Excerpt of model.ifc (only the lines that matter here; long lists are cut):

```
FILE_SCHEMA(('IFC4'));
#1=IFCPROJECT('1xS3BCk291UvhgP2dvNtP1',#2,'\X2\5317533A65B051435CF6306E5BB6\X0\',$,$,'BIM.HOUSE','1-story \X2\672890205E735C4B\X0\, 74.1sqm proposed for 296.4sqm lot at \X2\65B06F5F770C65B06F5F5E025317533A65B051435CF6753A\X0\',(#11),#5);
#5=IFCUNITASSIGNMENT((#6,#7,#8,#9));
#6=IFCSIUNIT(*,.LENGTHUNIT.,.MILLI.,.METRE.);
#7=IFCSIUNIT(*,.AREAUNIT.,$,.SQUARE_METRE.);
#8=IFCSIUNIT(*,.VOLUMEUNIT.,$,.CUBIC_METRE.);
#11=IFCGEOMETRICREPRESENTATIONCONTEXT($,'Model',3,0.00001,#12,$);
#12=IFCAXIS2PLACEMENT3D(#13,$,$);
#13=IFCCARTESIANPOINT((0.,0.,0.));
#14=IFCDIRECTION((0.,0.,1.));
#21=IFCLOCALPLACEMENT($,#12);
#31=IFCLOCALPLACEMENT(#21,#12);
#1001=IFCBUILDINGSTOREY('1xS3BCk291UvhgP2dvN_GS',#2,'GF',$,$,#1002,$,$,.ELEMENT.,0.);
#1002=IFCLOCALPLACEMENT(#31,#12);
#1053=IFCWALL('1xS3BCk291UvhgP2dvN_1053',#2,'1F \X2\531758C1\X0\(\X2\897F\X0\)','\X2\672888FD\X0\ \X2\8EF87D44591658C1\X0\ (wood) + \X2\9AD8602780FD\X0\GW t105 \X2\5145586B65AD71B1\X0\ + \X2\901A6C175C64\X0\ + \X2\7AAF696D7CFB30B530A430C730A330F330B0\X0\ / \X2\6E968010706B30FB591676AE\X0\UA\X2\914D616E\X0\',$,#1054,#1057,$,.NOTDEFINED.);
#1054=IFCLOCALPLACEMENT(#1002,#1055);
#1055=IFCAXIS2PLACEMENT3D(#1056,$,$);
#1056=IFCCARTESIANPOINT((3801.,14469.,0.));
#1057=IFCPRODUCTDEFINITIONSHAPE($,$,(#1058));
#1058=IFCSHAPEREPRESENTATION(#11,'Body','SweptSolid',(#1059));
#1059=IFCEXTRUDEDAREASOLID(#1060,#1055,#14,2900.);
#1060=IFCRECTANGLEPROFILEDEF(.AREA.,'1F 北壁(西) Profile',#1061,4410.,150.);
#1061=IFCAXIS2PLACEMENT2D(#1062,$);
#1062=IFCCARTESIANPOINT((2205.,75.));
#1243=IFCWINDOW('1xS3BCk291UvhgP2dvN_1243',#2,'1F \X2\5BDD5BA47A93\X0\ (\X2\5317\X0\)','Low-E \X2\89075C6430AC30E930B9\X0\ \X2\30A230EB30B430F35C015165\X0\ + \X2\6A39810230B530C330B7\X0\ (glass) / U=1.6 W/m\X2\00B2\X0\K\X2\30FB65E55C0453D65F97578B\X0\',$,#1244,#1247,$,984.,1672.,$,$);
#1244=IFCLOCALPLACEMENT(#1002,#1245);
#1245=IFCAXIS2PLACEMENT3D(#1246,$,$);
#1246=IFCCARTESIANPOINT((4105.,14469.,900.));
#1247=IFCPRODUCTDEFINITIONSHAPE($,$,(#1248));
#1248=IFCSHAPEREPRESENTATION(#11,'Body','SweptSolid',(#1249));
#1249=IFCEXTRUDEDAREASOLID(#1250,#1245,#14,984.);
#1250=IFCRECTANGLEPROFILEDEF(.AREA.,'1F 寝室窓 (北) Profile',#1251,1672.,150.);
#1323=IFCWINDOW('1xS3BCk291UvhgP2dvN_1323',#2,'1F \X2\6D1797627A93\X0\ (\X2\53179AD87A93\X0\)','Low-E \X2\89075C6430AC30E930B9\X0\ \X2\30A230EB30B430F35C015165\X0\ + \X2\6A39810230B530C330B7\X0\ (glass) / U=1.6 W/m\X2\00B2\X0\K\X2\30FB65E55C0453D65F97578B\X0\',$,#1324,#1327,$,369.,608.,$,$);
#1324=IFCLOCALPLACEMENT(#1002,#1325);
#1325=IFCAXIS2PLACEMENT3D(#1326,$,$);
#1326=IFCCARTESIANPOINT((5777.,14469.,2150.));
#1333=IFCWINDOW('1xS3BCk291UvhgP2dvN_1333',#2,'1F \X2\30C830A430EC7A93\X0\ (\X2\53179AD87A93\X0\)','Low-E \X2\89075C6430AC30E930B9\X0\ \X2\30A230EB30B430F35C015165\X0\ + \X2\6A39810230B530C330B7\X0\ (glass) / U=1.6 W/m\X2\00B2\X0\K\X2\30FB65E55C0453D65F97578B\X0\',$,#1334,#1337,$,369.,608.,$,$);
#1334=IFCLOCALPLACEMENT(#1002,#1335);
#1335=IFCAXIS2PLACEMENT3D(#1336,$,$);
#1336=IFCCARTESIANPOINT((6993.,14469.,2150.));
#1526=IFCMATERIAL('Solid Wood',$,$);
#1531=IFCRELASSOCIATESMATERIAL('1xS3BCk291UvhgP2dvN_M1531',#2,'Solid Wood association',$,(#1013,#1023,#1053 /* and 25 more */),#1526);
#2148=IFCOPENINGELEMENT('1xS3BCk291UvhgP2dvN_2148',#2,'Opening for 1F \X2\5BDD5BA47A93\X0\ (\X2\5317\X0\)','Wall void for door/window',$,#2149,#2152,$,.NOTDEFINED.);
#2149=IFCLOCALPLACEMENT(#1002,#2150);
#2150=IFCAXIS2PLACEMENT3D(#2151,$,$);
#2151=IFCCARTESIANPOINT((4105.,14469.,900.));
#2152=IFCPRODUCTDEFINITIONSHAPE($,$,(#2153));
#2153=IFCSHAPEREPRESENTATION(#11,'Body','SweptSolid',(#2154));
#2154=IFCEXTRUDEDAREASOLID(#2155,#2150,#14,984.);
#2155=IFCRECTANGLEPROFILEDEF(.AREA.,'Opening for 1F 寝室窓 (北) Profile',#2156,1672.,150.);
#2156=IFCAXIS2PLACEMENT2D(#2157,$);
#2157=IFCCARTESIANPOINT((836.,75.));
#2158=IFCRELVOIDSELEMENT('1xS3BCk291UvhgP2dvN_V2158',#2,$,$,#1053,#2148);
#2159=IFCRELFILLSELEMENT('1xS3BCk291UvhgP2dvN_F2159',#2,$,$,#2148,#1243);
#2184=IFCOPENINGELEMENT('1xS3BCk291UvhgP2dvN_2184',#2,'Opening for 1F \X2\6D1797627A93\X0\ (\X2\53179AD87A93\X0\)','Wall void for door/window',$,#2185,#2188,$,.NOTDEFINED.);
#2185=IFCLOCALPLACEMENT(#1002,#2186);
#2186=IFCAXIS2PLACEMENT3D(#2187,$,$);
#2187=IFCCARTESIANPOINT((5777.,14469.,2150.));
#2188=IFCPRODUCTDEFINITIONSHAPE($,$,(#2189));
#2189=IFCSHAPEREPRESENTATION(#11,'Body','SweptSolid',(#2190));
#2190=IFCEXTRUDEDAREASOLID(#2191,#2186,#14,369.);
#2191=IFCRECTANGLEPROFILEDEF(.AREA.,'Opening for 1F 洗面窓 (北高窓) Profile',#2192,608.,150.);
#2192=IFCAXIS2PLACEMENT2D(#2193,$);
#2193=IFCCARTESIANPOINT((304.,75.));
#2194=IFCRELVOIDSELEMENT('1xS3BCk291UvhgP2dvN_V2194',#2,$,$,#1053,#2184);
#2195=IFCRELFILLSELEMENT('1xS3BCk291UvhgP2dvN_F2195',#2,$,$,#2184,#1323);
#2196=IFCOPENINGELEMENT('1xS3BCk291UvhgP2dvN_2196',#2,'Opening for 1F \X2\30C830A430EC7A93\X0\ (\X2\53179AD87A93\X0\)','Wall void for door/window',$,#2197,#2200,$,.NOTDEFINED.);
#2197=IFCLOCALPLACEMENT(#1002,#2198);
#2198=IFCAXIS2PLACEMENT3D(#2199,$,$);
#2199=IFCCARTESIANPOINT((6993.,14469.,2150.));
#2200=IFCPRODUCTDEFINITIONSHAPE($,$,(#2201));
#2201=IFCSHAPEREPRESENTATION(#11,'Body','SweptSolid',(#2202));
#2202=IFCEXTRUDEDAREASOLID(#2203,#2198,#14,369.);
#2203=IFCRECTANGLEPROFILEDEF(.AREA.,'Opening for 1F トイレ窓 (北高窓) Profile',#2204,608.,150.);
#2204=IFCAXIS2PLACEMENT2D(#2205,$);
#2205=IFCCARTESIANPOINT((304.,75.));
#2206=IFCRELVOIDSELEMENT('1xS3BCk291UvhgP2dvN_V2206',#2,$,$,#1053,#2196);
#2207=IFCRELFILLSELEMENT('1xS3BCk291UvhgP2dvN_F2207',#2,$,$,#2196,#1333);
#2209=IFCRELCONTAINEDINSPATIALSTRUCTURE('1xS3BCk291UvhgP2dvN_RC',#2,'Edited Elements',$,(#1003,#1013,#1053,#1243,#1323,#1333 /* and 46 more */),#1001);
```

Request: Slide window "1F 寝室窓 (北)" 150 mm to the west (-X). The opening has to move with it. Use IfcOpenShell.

```python
import ifcopenshell
import ifcopenshell.api.geometry
import ifcopenshell.util.placement

model = ifcopenshell.open("model.ifc")

window = model.by_guid("1xS3BCk291UvhgP2dvN_1243")
opening = window.FillsVoids[0].RelatingOpeningElement
wall = opening.VoidsElements[0].RelatingBuildingElement

wall_matrix = ifcopenshell.util.placement.get_local_placement(wall.ObjectPlacement)
shift = wall_matrix[:3, 0] * -150.0
before = ifcopenshell.util.placement.get_local_placement(window.ObjectPlacement)[:3, 3].copy()

# The window is not placed relative to its opening, so move both.
for product in (opening, window):
    matrix = ifcopenshell.util.placement.get_local_placement(product.ObjectPlacement)
    matrix[:3, 3] += shift
    ifcopenshell.api.geometry.edit_object_placement(model, product=product, matrix=matrix, is_si=False)

after = ifcopenshell.util.placement.get_local_placement(window.ObjectPlacement)[:3, 3]
print("window moved by", (after - before).round(3) + 0.0)

model.write("model_rev.ifc")
```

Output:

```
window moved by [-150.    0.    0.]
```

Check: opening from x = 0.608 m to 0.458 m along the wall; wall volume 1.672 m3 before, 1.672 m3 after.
